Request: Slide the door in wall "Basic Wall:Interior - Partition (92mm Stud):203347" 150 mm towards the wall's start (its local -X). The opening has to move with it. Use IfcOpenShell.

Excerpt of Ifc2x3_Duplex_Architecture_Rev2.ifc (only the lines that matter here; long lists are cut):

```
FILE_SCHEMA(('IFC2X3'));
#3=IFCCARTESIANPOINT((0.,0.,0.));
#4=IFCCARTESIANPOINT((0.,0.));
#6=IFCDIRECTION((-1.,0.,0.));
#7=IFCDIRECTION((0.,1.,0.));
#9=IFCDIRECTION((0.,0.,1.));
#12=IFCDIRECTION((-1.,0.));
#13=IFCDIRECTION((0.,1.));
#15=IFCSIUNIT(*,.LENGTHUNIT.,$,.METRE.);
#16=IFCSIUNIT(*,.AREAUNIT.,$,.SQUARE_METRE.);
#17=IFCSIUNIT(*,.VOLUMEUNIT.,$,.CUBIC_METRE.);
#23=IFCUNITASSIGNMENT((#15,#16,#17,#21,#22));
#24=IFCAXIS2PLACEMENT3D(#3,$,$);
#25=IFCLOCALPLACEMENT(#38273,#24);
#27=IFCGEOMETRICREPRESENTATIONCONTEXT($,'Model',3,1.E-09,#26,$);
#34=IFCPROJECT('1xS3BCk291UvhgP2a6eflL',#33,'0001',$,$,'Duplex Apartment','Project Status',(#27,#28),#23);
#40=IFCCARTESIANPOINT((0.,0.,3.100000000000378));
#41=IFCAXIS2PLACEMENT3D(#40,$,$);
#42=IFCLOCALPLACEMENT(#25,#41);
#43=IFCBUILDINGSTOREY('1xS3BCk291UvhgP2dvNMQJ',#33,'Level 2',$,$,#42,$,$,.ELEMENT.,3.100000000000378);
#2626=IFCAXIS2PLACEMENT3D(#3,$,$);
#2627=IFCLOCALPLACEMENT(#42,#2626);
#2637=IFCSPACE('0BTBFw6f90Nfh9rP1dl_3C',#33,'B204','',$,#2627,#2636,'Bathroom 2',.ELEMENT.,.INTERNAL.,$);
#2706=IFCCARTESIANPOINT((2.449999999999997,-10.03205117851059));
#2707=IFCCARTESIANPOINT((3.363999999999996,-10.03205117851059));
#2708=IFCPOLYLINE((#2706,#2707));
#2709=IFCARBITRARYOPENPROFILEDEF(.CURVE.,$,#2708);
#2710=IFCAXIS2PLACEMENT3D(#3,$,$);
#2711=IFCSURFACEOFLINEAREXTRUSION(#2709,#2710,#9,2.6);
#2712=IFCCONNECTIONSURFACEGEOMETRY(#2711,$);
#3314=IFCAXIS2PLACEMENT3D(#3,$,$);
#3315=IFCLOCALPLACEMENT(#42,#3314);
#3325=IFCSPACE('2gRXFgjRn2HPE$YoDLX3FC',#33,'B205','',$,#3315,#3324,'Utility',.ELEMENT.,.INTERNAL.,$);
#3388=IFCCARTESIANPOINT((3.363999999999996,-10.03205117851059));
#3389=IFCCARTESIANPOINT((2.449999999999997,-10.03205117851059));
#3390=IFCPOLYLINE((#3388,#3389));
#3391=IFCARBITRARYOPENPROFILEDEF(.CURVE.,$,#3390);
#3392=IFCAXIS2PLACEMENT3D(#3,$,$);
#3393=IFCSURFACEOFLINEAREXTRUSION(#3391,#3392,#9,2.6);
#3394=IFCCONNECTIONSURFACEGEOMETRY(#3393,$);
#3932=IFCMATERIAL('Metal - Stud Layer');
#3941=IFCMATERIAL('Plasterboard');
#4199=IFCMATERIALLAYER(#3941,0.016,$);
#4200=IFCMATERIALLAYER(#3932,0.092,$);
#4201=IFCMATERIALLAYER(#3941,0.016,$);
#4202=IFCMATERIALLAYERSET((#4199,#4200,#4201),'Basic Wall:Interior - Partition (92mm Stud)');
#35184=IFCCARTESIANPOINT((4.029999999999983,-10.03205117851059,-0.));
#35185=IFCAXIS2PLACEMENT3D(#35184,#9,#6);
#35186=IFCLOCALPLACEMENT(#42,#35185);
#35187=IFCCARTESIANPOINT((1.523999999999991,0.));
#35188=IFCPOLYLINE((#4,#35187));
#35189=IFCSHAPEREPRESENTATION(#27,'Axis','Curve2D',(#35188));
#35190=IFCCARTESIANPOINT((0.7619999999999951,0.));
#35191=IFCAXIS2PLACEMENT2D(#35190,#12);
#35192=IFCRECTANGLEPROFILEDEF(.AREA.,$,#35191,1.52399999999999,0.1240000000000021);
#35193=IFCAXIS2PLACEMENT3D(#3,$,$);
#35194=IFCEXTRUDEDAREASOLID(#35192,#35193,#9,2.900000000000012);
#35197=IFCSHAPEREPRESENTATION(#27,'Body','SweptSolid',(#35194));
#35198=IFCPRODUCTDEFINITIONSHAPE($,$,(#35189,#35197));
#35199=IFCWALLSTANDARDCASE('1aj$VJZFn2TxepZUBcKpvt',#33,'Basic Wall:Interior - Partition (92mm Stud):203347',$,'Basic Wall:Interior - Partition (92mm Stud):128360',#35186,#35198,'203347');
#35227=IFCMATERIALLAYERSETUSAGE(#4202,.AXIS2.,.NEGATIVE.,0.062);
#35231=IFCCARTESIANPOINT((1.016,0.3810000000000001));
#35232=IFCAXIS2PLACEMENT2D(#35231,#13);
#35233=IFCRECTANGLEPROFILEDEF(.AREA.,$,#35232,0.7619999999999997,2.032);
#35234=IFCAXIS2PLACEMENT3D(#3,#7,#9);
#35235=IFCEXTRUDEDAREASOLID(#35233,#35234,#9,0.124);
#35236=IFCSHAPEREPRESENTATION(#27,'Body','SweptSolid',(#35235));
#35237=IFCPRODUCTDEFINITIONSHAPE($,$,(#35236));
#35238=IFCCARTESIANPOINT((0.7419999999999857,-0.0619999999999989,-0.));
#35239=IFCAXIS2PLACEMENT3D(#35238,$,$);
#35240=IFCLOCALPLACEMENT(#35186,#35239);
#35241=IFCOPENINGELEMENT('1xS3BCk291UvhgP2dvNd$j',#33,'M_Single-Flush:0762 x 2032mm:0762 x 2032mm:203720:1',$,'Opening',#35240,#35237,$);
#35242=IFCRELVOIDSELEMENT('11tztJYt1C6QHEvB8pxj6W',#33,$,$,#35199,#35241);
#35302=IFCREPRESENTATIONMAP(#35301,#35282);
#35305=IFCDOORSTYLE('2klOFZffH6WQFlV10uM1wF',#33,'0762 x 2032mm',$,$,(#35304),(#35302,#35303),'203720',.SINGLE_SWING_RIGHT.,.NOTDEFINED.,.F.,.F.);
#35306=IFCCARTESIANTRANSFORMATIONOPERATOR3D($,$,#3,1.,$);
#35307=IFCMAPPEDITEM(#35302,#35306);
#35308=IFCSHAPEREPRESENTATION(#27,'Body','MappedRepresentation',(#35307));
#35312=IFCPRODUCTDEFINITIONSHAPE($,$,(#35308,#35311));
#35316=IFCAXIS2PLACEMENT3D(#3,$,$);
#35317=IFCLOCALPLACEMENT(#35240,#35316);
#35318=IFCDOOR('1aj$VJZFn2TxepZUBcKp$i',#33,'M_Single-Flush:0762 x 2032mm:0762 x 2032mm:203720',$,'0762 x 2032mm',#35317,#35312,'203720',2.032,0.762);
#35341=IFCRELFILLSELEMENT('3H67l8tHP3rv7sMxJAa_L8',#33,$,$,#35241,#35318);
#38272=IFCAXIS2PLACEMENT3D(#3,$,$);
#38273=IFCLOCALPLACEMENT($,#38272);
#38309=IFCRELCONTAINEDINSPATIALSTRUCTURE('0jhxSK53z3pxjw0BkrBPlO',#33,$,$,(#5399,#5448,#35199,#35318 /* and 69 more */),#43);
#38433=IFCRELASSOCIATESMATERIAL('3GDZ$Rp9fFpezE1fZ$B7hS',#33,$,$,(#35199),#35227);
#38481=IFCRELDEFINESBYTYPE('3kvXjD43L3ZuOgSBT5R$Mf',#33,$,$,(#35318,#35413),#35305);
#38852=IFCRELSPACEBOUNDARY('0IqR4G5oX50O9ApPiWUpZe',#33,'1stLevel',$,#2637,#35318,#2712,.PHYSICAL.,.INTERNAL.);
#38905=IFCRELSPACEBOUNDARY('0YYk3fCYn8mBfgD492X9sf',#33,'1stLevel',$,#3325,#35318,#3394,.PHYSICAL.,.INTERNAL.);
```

```python
import numpy as np
import ifcopenshell
import ifcopenshell.api.geometry
import ifcopenshell.util.placement
import ifcopenshell.util.unit

model = ifcopenshell.open("Ifc2x3_Duplex_Architecture_Rev2.ifc")
unit_scale = ifcopenshell.util.unit.calculate_unit_scale(model)

door = model.by_guid("1aj$VJZFn2TxepZUBcKp$i")
opening = door.FillsVoids[0].RelatingOpeningElement
wall = opening.VoidsElements[0].RelatingBuildingElement

wall_matrix = ifcopenshell.util.placement.get_local_placement(wall.ObjectPlacement)
shift = wall_matrix[:3, 0] * -0.15 / unit_scale
before = ifcopenshell.util.placement.get_local_placement(door.ObjectPlacement)[:3, 3].copy()

# The door is placed relative to its opening, so it follows when the opening moves.
matrix = ifcopenshell.util.placement.get_local_placement(opening.ObjectPlacement)
matrix[:3, 3] += shift
ifcopenshell.api.geometry.edit_object_placement(
    model, product=opening, matrix=matrix, is_si=False, should_transform_children=True
)

# Space boundary surfaces are stored in each space's coordinates; move them too.
for rel in door.ProvidesBoundaries:
    if not rel.ConnectionGeometry:
        continue
    surface = rel.ConnectionGeometry.SurfaceOnRelatingElement
    space_matrix = ifcopenshell.util.placement.get_local_placement(rel.RelatingSpace.ObjectPlacement)
    point = np.array(surface.Position.Location.Coordinates) + space_matrix[:3, :3].T @ shift
    surface.Position = model.createIfcAxis2Placement3D(
        model.createIfcCartesianPoint(point.tolist()), surface.Position.Axis, surface.Position.RefDirection
    )

after = ifcopenshell.util.placement.get_local_placement(door.ObjectPlacement)[:3, 3]
print("door moved by", (after - before).round(3) + 0.0)

model.write("Ifc2x3_Duplex_Architecture_Rev2-out.ifc")
```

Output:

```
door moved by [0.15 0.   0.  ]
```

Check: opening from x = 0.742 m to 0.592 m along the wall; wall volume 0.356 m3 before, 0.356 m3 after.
